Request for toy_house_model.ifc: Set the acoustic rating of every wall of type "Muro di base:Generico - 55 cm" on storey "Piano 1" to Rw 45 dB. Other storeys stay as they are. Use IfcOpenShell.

First a look at what the model holds.

```python
import ifcopenshell
import ifcopenshell.util.element

model = ifcopenshell.open("toy_house_model.ifc")
print(model.schema)
storey = next(s for s in model.by_type("IfcBuildingStorey") if s.Name == "Piano 1")
walls = [e for e in ifcopenshell.util.element.get_decomposition(storey) if e.is_a("IfcWall")]
seen = {}
for e in walls:
    element_type = ifcopenshell.util.element.get_type(e)
    key = (element_type.Name if element_type != e and element_type else None, ifcopenshell.util.element.get_pset(e, "Pset_WallCommon", "AcousticRating"))
    seen[key] = seen.get(key, 0) + 1
for (name, value), count in sorted(seen.items(), key=str):
    print(count, "x", name, "|", value)
```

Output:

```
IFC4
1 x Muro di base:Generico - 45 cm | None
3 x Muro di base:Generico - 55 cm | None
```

```python
import ifcopenshell
import ifcopenshell.api.pset
import ifcopenshell.util.element

model = ifcopenshell.open("toy_house_model.ifc")

storey = next(s for s in model.by_type("IfcBuildingStorey") if s.Name == "Piano 1")
walls = [e for e in ifcopenshell.util.element.get_decomposition(storey) if e.is_a("IfcWall")]

count = 0
for e in walls:
    element_type = ifcopenshell.util.element.get_type(e)
    if element_type in (None, e) or element_type.Name != "Muro di base:Generico - 55 cm":
        continue
    # add_pset returns the element's existing set when there is one.
    pset = ifcopenshell.api.pset.add_pset(model, product=e, name="Pset_WallCommon")
    ifcopenshell.api.pset.edit_pset(model, pset=pset, properties={"AcousticRating": "Rw 45 dB"})
    count += 1

print(count, "walls updated")

model.write("toy_house_model_updated.ifc")
```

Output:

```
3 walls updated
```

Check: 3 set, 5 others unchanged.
